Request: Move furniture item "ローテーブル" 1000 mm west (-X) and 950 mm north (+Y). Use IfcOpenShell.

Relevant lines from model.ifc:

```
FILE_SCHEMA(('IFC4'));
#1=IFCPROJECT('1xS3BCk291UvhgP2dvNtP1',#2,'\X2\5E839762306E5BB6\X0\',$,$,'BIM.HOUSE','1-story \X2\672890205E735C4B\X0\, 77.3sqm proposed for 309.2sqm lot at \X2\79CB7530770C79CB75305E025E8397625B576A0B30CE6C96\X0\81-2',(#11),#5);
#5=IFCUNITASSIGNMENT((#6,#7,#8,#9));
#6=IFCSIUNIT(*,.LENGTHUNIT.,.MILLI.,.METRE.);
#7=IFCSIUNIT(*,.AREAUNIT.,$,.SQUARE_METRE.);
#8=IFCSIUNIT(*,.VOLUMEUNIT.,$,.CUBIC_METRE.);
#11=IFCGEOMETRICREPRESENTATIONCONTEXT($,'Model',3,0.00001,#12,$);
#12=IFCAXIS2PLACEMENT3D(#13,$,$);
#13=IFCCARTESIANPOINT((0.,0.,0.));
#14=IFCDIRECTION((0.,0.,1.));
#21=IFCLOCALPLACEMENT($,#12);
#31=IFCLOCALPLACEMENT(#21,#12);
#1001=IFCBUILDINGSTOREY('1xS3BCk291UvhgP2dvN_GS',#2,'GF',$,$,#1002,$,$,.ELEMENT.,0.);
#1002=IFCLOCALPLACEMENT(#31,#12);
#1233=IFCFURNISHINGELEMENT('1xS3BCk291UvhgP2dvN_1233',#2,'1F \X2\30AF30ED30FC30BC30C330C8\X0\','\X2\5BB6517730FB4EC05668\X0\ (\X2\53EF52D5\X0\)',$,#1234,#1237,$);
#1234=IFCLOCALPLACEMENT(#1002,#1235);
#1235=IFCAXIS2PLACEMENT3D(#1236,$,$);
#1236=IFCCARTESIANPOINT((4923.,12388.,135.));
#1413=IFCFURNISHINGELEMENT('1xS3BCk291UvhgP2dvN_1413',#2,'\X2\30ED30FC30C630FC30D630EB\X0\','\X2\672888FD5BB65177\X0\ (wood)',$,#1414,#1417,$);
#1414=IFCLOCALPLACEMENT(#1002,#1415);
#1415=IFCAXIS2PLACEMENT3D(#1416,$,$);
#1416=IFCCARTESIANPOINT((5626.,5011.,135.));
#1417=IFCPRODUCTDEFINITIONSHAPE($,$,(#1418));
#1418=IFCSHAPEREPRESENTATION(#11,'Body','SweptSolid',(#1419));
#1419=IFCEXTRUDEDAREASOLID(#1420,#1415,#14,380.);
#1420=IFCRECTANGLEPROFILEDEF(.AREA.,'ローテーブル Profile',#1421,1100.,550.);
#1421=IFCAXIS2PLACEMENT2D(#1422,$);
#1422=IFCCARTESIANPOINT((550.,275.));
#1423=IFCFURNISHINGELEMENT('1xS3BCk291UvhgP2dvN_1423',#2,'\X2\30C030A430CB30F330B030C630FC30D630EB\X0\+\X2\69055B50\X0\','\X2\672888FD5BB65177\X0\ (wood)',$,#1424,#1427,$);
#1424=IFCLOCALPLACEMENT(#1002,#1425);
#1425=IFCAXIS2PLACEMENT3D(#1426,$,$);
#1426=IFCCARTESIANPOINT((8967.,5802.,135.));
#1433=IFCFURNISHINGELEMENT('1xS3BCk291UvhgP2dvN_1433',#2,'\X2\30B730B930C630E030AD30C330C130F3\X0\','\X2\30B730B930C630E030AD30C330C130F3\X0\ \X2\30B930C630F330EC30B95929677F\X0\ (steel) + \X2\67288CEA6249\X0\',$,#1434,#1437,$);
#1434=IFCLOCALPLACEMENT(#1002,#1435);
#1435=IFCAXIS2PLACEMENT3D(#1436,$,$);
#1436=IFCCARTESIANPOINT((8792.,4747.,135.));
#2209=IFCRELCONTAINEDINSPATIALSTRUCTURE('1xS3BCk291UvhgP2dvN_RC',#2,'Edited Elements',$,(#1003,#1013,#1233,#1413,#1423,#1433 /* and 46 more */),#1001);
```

```python
import ifcopenshell
import ifcopenshell.api.geometry
import ifcopenshell.util.placement
import ifcopenshell.util.unit

model = ifcopenshell.open("model.ifc")
unit_scale = ifcopenshell.util.unit.calculate_unit_scale(model)

item = model.by_id(1413)
matrix = ifcopenshell.util.placement.get_local_placement(item.ObjectPlacement)
matrix[0, 3] -= 1 / unit_scale
matrix[1, 3] += 0.95 / unit_scale
ifcopenshell.api.geometry.edit_object_placement(model, product=item, matrix=matrix, is_si=False)

print(ifcopenshell.util.placement.get_local_placement(item.ObjectPlacement).round(3) + 0.0)

model.write("model_edited.ifc")
```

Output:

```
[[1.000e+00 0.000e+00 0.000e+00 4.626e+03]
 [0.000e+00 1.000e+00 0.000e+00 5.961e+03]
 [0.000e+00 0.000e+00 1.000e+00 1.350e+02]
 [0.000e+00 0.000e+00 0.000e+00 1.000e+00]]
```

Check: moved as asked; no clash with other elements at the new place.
